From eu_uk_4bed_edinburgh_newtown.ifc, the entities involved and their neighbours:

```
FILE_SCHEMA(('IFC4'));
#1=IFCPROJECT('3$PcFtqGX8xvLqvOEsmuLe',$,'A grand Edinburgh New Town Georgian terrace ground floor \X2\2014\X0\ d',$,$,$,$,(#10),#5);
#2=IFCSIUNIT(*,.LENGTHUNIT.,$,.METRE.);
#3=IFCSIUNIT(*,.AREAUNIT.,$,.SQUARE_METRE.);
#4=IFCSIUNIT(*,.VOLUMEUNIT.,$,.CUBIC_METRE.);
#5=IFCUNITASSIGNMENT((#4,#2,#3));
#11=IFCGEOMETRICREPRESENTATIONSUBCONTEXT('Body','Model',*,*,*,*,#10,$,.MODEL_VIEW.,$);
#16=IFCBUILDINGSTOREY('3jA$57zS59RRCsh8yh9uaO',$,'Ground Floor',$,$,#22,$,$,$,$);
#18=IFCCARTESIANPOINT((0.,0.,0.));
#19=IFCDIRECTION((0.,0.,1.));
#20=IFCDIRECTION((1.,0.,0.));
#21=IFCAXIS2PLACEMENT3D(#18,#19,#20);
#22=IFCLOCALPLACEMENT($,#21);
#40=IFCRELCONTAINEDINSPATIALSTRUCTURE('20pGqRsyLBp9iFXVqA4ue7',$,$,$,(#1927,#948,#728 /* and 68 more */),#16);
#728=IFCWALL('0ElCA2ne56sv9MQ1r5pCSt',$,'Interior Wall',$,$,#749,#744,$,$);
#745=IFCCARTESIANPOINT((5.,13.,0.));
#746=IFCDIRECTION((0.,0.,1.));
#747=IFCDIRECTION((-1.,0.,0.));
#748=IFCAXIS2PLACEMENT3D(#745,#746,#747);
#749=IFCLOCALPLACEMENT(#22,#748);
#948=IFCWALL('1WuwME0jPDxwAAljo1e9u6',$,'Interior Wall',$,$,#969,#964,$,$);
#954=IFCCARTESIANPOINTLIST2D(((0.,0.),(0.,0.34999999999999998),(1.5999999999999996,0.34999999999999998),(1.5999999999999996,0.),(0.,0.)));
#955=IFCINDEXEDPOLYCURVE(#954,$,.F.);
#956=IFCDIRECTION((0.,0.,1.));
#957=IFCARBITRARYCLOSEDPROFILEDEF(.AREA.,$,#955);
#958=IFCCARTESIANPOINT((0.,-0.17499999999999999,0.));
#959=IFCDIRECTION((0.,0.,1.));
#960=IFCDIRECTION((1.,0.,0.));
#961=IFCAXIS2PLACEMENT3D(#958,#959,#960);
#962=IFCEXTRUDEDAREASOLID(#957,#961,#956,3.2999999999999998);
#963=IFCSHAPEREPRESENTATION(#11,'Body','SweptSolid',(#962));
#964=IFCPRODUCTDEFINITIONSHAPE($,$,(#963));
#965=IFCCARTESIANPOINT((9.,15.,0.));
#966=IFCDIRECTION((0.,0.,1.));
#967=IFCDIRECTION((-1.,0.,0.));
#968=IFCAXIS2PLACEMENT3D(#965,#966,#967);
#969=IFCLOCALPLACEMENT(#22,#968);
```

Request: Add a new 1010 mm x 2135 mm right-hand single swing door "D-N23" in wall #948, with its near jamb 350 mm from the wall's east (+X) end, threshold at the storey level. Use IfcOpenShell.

```python
import numpy as np
import ifcopenshell
import ifcopenshell.api.feature
import ifcopenshell.api.geometry
import ifcopenshell.api.root
import ifcopenshell.api.spatial
import ifcopenshell.geom
import ifcopenshell.util.element
import ifcopenshell.util.placement
import ifcopenshell.util.representation
import ifcopenshell.util.shape
import ifcopenshell.util.unit

model = ifcopenshell.open("eu_uk_4bed_edinburgh_newtown.ifc")
unit_scale = ifcopenshell.util.unit.calculate_unit_scale(model)
settings = ifcopenshell.geom.settings()


def volume(element):
    """Net volume in cubic metres, openings subtracted."""
    shape = ifcopenshell.geom.create_shape(settings, element)
    return ifcopenshell.util.shape.get_volume(shape.geometry)


wall = model.by_guid("1WuwME0jPDxwAAljo1e9u6")
storey = ifcopenshell.util.element.get_container(wall, ifc_class="IfcBuildingStorey")
context = ifcopenshell.util.representation.get_context(model, "Model", "Body", "MODEL_VIEW")
before = volume(wall)

width, height, from_end, sill = 1.01, 2.135, 0.35, 0.0  # metres

# The wall runs along its own X axis, and the end named is its -X end.
wall_shape = ifcopenshell.geom.create_shape(settings, wall)
x, y, z = ifcopenshell.util.shape.get_vertices(wall_shape.geometry).T
start = x.min() + from_end
face, thickness = float(y.min()), float(y.max() - y.min())
wall_matrix = ifcopenshell.util.placement.get_local_placement(wall.ObjectPlacement)
level = ifcopenshell.util.placement.get_local_placement(storey.ObjectPlacement)[2, 3]


def in_wall(x, y):
    """Placement at x, y metres in the wall's axes, at sill height."""
    matrix = wall_matrix.copy()
    matrix[:, 3] = wall_matrix @ np.array([x / unit_scale, y / unit_scale, 0.0, 1.0])
    matrix[2, 3] = level + sill / unit_scale
    return matrix


# Opening: a box that overshoots both wall faces by 50 mm.
opening = ifcopenshell.api.root.create_entity(model, ifc_class="IfcOpeningElement", predefined_type="OPENING")
box = ifcopenshell.api.geometry.add_wall_representation(
    model, context=context, length=width, height=height, thickness=thickness + 0.1
)
ifcopenshell.api.geometry.assign_representation(model, product=opening, representation=box)
ifcopenshell.api.geometry.edit_object_placement(model, product=opening, matrix=in_wall(start, face - 0.05), is_si=False)
ifcopenshell.api.feature.add_feature(model, feature=opening, element=wall)

door = ifcopenshell.api.root.create_entity(model, ifc_class="IfcDoor", name="D-N23", predefined_type="DOOR")
door.OverallWidth, door.OverallHeight = width / unit_scale, height / unit_scale
door.OperationType = "SINGLE_SWING_RIGHT"
body = ifcopenshell.api.geometry.add_door_representation(
    model,
    context=context,
    overall_width=door.OverallWidth,
    overall_height=door.OverallHeight,
    operation_type="SINGLE_SWING_RIGHT",
    lining_properties={"LiningDepth": thickness / unit_scale, "ThresholdDepth": thickness / unit_scale},
)
ifcopenshell.api.geometry.assign_representation(model, product=door, representation=body)
ifcopenshell.api.spatial.assign_container(model, products=[door], relating_structure=storey)
ifcopenshell.api.feature.add_filling(model, opening=opening, element=door)

# The lining spans the wall, so the door starts at the wall face.
ifcopenshell.api.geometry.edit_object_placement(model, product=door, matrix=in_wall(start, face), is_si=False)

after = volume(wall)

print(f"wall volume {before:.3f} -> {after:.3f} m3")

model.write("eu_uk_4bed_edinburgh_newtown_rev.ifc")
```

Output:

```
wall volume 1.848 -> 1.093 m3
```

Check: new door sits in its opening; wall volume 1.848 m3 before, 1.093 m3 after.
